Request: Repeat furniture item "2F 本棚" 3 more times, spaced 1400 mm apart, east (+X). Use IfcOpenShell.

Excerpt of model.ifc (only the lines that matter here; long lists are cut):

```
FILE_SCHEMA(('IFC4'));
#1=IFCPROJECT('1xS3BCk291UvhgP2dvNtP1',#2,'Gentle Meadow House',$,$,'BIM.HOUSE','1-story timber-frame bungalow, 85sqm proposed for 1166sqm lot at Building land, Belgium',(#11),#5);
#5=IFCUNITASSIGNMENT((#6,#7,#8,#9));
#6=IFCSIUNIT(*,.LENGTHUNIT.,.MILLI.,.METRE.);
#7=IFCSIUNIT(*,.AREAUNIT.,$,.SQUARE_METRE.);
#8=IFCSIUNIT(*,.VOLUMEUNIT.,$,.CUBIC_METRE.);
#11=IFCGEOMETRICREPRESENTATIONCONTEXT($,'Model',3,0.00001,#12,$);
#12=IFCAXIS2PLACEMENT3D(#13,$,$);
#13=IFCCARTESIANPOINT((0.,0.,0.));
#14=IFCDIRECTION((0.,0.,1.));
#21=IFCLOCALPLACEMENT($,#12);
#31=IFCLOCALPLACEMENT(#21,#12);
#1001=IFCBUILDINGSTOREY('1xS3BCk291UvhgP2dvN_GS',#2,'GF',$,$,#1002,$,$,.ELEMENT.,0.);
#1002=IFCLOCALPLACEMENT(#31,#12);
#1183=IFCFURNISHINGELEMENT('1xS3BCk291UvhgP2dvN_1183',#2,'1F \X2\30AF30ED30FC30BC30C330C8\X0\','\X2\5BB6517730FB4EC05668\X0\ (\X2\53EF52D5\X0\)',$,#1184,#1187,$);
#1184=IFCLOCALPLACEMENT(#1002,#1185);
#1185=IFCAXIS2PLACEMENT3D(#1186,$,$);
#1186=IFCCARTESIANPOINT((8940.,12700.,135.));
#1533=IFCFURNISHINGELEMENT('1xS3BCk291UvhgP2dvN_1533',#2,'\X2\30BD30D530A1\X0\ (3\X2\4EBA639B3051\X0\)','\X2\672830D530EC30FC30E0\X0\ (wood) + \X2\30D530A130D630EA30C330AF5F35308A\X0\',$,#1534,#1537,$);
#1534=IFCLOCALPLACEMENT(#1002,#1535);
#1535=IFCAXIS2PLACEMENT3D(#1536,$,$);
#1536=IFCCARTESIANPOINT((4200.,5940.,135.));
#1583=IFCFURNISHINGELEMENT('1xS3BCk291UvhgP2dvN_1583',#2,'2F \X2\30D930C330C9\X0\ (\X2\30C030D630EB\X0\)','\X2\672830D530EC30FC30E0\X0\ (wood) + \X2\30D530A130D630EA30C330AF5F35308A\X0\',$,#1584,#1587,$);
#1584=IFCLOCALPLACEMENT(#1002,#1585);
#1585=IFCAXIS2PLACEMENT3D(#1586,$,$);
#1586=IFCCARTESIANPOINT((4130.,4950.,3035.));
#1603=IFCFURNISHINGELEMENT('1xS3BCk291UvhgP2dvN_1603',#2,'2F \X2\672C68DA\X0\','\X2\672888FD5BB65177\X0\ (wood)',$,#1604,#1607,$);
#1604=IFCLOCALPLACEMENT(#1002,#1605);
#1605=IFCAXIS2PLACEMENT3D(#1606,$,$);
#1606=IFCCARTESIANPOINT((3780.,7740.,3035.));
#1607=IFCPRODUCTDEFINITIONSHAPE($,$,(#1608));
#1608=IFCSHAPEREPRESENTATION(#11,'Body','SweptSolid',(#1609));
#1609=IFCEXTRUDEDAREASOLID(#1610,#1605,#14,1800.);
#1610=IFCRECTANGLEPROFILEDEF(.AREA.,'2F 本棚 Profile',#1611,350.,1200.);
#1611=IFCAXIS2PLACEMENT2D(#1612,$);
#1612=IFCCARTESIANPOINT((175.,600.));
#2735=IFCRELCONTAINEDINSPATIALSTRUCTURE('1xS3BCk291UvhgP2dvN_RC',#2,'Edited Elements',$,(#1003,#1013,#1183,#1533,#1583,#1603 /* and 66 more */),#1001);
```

```python
import numpy as np
import ifcopenshell
import ifcopenshell.api.geometry
import ifcopenshell.api.root
import ifcopenshell.util.element
import ifcopenshell.util.placement
import ifcopenshell.util.unit

model = ifcopenshell.open("model.ifc")
unit_scale = ifcopenshell.util.unit.calculate_unit_scale(model)


def reuse_history(source, copy):
    """copy_class also copies each property set's owner history, people and application; keep the originals."""
    for rel in copy.IsDefinedBy:
        if rel.is_a("IfcRelDefinesByProperties") and (history := rel.RelatingPropertyDefinition.OwnerHistory):
            rel.RelatingPropertyDefinition.OwnerHistory = source.OwnerHistory
            ifcopenshell.util.element.remove_deep2(model, history)


source = model.by_guid("1xS3BCk291UvhgP2dvN_1603")
base = ifcopenshell.util.placement.get_local_placement(source.ObjectPlacement)
step = np.array([1.0, 0.0, 0.0]) * 1.4 / unit_scale

for i in range(1, 4):
    copy = ifcopenshell.api.root.copy_class(model, product=source)
    copy.Representation = ifcopenshell.util.element.copy_deep(
        model, source.Representation, exclude=["IfcGeometricRepresentationContext", "IfcRepresentationMap"]
    )
    reuse_history(source, copy)
    matrix = base.copy()
    matrix[:3, 3] += i * step
    print("added at", matrix[:3, 3].round(3) + 0.0)
    ifcopenshell.api.geometry.edit_object_placement(model, product=copy, matrix=matrix, is_si=False)

model.write("model-out.ifc")
```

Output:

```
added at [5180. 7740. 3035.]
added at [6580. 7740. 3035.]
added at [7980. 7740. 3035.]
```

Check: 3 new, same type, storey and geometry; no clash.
